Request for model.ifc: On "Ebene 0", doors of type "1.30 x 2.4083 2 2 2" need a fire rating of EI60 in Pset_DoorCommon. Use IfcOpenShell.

First a look at what the model holds.

```python
import ifcopenshell
import ifcopenshell.util.element

model = ifcopenshell.open("model.ifc")
print(model.schema)
storey = next(s for s in model.by_type("IfcBuildingStorey") if s.Name == "Ebene 0")
doors = [e for e in ifcopenshell.util.element.get_decomposition(storey) if e.is_a("IfcDoor")]
seen = {}
for e in doors:
    element_type = ifcopenshell.util.element.get_type(e)
    key = (element_type.Name if element_type != e and element_type else None, ifcopenshell.util.element.get_pset(e, "Pset_DoorCommon", "FireRating"))
    seen[key] = seen.get(key, 0) + 1
for (name, value), count in sorted(seen.items(), key=str):
    print(count, "x", name, "|", value)
```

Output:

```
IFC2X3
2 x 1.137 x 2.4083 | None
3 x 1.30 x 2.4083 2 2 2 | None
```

```python
import ifcopenshell
import ifcopenshell.api.pset
import ifcopenshell.util.element

model = ifcopenshell.open("model.ifc")

storey = next(s for s in model.by_type("IfcBuildingStorey") if s.Name == "Ebene 0")
doors = [e for e in ifcopenshell.util.element.get_decomposition(storey) if e.is_a("IfcDoor")]

count = 0
for e in doors:
    element_type = ifcopenshell.util.element.get_type(e)
    if element_type in (None, e) or element_type.Name != "1.30 x 2.4083 2 2 2":
        continue
    # add_pset returns the element's existing set when there is one.
    pset = ifcopenshell.api.pset.add_pset(model, product=e, name="Pset_DoorCommon")
    ifcopenshell.api.pset.edit_pset(model, pset=pset, properties={"FireRating": "EI60"})
    count += 1

print(count, "doors updated")

model.write("model_updated.ifc")
```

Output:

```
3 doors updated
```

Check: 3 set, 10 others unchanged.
